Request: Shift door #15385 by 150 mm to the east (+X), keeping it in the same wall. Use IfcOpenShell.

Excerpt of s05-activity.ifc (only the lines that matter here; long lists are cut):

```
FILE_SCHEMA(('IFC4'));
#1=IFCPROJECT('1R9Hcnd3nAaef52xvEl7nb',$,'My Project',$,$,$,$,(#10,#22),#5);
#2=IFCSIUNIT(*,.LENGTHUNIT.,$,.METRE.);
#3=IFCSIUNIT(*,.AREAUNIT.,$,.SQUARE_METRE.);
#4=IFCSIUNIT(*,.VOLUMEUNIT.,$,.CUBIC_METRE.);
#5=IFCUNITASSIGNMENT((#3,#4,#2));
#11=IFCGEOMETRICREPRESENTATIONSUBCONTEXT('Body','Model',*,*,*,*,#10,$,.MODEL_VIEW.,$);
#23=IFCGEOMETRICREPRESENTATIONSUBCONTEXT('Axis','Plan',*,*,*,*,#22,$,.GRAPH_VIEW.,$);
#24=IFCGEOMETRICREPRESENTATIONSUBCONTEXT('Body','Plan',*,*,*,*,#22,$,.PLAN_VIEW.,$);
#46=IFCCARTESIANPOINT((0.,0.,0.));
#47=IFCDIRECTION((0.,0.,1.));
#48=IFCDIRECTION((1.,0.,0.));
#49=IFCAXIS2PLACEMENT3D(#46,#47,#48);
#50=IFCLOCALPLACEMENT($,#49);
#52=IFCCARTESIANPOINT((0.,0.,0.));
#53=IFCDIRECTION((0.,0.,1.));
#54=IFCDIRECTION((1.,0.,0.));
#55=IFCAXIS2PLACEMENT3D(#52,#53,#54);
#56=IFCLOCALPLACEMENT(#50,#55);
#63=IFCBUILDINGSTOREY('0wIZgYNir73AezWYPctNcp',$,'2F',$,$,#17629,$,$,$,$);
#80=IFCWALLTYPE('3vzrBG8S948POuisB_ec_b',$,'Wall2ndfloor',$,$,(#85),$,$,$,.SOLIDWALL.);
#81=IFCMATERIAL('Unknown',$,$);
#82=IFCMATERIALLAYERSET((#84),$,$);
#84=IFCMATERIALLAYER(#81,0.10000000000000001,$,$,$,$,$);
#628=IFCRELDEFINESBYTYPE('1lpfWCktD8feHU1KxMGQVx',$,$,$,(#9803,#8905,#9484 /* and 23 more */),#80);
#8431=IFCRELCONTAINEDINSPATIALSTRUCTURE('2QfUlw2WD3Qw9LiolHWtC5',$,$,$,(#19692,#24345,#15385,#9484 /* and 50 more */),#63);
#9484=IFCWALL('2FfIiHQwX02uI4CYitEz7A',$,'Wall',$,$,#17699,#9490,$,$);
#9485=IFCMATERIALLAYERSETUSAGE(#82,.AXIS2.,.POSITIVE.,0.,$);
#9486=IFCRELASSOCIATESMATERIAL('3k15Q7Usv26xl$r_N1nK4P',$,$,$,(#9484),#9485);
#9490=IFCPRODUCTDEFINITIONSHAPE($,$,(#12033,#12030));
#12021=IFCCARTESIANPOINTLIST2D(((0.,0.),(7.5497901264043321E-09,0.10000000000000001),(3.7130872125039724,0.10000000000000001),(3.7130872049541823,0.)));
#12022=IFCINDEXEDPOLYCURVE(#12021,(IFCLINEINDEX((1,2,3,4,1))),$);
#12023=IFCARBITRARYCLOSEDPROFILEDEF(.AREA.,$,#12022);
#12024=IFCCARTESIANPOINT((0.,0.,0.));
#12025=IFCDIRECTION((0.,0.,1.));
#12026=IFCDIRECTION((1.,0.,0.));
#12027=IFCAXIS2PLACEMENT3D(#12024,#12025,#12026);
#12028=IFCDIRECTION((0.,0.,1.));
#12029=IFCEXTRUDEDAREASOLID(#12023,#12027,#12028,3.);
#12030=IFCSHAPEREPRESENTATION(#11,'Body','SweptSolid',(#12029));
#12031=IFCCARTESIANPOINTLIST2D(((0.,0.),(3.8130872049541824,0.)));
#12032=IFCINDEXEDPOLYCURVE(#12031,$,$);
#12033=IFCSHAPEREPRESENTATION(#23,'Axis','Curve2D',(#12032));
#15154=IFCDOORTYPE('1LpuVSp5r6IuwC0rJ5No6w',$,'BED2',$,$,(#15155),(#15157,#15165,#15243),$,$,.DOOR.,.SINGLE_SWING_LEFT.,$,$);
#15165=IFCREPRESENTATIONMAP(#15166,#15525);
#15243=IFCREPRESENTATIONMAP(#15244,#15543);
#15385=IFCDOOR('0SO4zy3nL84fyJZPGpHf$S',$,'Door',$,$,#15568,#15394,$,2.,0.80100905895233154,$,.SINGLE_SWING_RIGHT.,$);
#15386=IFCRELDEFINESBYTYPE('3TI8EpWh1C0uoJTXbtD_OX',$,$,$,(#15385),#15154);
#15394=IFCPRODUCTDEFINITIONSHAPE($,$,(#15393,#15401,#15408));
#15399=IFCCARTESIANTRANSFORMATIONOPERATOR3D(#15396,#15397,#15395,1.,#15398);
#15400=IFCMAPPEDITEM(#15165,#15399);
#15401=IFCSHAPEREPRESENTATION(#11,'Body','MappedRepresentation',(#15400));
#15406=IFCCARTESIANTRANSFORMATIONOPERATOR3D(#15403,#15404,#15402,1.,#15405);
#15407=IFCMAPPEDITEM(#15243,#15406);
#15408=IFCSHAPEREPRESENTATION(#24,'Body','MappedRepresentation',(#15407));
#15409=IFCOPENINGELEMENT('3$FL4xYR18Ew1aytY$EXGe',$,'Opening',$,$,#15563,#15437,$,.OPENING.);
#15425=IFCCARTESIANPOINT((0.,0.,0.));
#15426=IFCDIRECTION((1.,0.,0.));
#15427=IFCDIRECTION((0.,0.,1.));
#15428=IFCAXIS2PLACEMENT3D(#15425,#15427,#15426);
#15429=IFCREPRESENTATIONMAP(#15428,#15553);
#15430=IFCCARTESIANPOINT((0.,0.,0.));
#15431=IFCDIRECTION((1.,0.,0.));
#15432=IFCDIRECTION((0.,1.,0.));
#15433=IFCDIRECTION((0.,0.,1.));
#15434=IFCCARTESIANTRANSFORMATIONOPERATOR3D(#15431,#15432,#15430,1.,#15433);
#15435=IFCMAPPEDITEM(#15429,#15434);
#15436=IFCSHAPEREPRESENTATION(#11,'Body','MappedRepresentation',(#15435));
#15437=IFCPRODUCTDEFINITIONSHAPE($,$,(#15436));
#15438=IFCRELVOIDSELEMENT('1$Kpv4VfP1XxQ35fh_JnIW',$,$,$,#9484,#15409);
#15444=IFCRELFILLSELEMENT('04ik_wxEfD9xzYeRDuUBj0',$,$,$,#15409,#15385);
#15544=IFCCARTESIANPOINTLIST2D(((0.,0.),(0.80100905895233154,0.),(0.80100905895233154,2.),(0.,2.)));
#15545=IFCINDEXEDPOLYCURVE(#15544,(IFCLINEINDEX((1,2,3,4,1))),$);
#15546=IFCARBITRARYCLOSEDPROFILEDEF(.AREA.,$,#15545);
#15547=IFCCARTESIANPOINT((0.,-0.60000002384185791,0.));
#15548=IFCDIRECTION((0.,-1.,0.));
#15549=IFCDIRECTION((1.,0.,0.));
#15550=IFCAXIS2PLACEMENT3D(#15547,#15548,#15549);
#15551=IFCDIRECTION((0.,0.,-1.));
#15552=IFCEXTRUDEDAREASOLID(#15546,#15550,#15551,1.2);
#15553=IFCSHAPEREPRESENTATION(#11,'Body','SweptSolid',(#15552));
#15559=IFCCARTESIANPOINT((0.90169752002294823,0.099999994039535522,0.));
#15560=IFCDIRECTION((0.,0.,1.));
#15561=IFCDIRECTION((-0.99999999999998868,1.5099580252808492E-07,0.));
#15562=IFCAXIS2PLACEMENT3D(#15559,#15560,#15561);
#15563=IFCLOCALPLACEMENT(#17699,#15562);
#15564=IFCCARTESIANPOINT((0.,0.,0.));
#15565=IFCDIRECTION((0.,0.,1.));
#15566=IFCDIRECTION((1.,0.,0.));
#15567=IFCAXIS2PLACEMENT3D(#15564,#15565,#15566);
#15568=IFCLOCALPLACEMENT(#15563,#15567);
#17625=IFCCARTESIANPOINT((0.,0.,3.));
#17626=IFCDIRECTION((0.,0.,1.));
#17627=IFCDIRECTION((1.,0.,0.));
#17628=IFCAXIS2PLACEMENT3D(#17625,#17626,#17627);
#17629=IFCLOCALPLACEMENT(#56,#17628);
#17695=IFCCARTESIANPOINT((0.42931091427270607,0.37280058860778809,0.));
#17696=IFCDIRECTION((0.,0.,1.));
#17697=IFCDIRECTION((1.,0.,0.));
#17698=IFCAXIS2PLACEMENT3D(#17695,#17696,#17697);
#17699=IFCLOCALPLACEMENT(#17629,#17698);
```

```python
import ifcopenshell
import ifcopenshell.api.geometry
import ifcopenshell.util.placement
import ifcopenshell.util.unit

model = ifcopenshell.open("s05-activity.ifc")
unit_scale = ifcopenshell.util.unit.calculate_unit_scale(model)

door = model.by_id(15385)
opening = door.FillsVoids[0].RelatingOpeningElement
wall = opening.VoidsElements[0].RelatingBuildingElement

wall_matrix = ifcopenshell.util.placement.get_local_placement(wall.ObjectPlacement)
shift = wall_matrix[:3, 0] * 0.15 / unit_scale
before = ifcopenshell.util.placement.get_local_placement(door.ObjectPlacement)[:3, 3].copy()

# The door is placed relative to its opening, so it follows when the opening moves.
matrix = ifcopenshell.util.placement.get_local_placement(opening.ObjectPlacement)
matrix[:3, 3] += shift
ifcopenshell.api.geometry.edit_object_placement(
    model, product=opening, matrix=matrix, is_si=False, should_transform_children=True
)

after = ifcopenshell.util.placement.get_local_placement(door.ObjectPlacement)[:3, 3]
print("door moved by", (after - before).round(3) + 0.0)

model.write("s05-activity_rev.ifc")
```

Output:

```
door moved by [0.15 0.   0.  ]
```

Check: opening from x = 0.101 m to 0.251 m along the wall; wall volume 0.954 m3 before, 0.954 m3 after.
